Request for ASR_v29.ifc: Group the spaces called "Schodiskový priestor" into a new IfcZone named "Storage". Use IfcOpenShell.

First a look at what the model holds.

```python
import ifcopenshell

model = ifcopenshell.open("ASR_v29.ifc")
print(model.schema)
seen = {}
for space in model.by_type("IfcSpace"):
    seen[space.LongName] = seen.get(space.LongName, 0) + 1
for name, count in sorted(seen.items(), key=str):
    print(count, "x", name)
print("zones:", [z.Name for z in model.by_type("IfcZone")][:20])
```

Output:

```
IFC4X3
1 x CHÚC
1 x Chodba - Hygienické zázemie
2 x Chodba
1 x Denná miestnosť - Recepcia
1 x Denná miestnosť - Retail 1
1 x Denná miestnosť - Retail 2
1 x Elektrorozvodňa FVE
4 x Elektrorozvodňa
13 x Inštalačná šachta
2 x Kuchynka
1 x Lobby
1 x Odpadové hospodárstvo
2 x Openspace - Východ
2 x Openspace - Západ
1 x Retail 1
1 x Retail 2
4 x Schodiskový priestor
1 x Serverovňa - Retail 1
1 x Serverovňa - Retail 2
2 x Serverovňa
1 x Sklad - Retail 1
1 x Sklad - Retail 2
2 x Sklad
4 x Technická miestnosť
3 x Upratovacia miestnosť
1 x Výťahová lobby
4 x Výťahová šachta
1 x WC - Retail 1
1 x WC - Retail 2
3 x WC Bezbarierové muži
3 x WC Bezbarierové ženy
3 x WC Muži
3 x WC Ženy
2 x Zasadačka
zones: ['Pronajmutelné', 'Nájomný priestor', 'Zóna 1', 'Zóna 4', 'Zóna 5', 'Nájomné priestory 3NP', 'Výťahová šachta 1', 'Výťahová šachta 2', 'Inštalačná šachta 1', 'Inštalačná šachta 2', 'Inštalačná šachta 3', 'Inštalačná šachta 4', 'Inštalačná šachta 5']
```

```python
import ifcopenshell
import ifcopenshell.api.group
import ifcopenshell.api.root

model = ifcopenshell.open("ASR_v29.ifc")

names = {"Schodiskový priestor"}
spaces = [s for s in model.by_type("IfcSpace") if s.LongName in names]

zone = ifcopenshell.api.root.create_entity(model, ifc_class="IfcZone", name="Storage")
ifcopenshell.api.group.assign_group(model, products=spaces, group=zone)
print(len(spaces), "spaces in", zone.Name)

model.write("ASR_v29_updated.ifc")
```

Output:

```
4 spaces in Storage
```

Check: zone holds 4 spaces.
